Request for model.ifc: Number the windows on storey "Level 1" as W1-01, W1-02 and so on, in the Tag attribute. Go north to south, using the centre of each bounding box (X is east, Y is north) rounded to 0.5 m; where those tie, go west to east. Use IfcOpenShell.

First a look at what the model holds.

```python
import ifcopenshell
import ifcopenshell.util.element
import ifcopenshell.util.placement

model = ifcopenshell.open("model.ifc")
print(model.schema)
storey = next(s for s in model.by_type("IfcBuildingStorey") if s.Name == "Level 1")
windows = [e for e in ifcopenshell.util.element.get_decomposition(storey) if e.is_a("IfcWindow")]
for e in sorted(windows, key=lambda e: e.id()):
    origin = ifcopenshell.util.placement.get_local_placement(e.ObjectPlacement)[:3, 3]
    print(e.id(), e.Tag, e.Name, origin.round(2) + 0.0, sep=" | ")
```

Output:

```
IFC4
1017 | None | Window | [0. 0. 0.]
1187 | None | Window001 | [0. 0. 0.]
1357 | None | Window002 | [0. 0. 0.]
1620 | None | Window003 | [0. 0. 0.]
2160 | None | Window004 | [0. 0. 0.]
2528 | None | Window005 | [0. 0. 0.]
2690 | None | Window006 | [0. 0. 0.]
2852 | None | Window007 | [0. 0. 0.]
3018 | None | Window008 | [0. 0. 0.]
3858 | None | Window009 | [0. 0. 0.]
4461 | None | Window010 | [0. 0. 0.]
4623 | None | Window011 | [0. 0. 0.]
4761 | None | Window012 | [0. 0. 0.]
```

```python
import ifcopenshell
import ifcopenshell.geom
import ifcopenshell.util.element
import ifcopenshell.util.shape

model = ifcopenshell.open("model.ifc")
settings = ifcopenshell.geom.settings()
settings.set("use-world-coords", True)


def centre(element):
    shape = ifcopenshell.geom.create_shape(settings, element)
    return ifcopenshell.util.shape.get_bbox_centroid(shape.geometry)


storey = next(s for s in model.by_type("IfcBuildingStorey") if s.Name == "Level 1")
windows = [e for e in ifcopenshell.util.element.get_decomposition(storey) if e.is_a("IfcWindow")]

# Insertion points can sit at a corner or the storey origin, so sort by the geometry (in metres).
centres = {e: centre(e) for e in windows}
windows.sort(key=lambda e: (-round(centres[e][1] / 0.5), centres[e][0]))

for i, e in enumerate(windows, start=1):
    number = f"W1-{i:02d}"
    e.Tag = number
    print(e.id(), number)

model.write("model_updated.ifc")
```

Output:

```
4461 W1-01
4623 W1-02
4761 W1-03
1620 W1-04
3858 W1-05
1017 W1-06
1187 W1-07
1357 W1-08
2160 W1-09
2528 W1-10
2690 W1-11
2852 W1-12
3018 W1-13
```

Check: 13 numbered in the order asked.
